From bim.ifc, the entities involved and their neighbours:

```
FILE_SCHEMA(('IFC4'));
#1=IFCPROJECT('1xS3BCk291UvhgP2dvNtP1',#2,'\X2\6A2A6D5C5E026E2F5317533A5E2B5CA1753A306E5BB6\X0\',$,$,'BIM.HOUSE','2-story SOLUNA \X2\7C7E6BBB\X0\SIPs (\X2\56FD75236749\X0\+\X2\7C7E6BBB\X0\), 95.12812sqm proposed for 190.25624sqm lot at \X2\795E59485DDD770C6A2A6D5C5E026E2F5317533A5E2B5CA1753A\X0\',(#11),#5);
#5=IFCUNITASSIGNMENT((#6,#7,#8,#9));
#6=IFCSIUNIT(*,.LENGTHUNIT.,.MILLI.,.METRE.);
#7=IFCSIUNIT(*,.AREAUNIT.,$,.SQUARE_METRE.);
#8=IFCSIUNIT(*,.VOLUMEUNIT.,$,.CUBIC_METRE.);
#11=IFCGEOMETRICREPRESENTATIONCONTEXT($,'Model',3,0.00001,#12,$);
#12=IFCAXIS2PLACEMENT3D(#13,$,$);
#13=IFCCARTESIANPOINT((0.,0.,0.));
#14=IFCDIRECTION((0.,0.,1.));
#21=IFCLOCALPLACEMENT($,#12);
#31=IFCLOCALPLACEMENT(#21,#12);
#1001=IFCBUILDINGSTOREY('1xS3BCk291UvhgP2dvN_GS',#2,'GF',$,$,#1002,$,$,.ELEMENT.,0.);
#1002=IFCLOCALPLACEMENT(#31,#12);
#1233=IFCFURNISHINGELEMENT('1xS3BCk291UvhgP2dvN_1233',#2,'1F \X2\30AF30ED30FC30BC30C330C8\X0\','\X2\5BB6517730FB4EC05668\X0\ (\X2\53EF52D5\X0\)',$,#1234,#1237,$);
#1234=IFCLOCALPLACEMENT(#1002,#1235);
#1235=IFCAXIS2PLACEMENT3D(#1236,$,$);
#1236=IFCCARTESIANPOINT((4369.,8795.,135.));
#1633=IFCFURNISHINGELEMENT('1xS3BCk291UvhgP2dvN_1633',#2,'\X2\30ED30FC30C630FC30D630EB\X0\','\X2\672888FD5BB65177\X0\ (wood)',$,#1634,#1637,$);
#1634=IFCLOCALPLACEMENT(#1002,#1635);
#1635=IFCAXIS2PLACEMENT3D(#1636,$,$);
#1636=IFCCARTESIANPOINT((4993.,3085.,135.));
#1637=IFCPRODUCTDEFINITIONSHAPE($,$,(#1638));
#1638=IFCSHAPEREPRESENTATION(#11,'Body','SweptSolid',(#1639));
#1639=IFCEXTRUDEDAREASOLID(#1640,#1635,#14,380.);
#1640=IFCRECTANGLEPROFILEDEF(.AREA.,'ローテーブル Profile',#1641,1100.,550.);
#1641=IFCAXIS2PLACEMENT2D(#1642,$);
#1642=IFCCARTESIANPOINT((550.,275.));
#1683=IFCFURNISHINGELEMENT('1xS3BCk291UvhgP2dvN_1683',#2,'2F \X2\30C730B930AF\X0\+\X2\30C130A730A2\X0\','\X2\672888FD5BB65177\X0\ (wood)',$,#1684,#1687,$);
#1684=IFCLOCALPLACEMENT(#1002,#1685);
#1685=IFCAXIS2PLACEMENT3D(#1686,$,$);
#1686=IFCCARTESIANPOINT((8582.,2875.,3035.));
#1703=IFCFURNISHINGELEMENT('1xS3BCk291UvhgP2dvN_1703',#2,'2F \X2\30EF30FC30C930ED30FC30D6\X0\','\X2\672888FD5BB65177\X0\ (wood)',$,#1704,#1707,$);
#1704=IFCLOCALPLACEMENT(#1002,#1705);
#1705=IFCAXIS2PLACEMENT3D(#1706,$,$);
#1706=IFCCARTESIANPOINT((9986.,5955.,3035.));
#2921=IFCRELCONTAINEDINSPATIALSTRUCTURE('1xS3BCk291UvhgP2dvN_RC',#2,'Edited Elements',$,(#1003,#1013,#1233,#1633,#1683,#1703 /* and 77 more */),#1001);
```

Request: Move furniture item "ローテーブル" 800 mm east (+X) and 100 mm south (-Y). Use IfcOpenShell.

```python
import ifcopenshell
import ifcopenshell.api.geometry
import ifcopenshell.util.placement
import ifcopenshell.util.unit

model = ifcopenshell.open("bim.ifc")
unit_scale = ifcopenshell.util.unit.calculate_unit_scale(model)

item = model.by_guid("1xS3BCk291UvhgP2dvN_1633")
matrix = ifcopenshell.util.placement.get_local_placement(item.ObjectPlacement)
matrix[0, 3] += 0.8 / unit_scale
matrix[1, 3] -= 0.1 / unit_scale
ifcopenshell.api.geometry.edit_object_placement(model, product=item, matrix=matrix, is_si=False)

print(ifcopenshell.util.placement.get_local_placement(item.ObjectPlacement).round(3) + 0.0)

model.write("bim_edited.ifc")
```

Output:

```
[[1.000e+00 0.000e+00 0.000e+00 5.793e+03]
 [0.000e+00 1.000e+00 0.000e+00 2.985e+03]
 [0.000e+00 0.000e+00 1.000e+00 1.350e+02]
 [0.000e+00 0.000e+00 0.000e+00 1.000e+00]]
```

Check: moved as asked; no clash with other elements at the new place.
